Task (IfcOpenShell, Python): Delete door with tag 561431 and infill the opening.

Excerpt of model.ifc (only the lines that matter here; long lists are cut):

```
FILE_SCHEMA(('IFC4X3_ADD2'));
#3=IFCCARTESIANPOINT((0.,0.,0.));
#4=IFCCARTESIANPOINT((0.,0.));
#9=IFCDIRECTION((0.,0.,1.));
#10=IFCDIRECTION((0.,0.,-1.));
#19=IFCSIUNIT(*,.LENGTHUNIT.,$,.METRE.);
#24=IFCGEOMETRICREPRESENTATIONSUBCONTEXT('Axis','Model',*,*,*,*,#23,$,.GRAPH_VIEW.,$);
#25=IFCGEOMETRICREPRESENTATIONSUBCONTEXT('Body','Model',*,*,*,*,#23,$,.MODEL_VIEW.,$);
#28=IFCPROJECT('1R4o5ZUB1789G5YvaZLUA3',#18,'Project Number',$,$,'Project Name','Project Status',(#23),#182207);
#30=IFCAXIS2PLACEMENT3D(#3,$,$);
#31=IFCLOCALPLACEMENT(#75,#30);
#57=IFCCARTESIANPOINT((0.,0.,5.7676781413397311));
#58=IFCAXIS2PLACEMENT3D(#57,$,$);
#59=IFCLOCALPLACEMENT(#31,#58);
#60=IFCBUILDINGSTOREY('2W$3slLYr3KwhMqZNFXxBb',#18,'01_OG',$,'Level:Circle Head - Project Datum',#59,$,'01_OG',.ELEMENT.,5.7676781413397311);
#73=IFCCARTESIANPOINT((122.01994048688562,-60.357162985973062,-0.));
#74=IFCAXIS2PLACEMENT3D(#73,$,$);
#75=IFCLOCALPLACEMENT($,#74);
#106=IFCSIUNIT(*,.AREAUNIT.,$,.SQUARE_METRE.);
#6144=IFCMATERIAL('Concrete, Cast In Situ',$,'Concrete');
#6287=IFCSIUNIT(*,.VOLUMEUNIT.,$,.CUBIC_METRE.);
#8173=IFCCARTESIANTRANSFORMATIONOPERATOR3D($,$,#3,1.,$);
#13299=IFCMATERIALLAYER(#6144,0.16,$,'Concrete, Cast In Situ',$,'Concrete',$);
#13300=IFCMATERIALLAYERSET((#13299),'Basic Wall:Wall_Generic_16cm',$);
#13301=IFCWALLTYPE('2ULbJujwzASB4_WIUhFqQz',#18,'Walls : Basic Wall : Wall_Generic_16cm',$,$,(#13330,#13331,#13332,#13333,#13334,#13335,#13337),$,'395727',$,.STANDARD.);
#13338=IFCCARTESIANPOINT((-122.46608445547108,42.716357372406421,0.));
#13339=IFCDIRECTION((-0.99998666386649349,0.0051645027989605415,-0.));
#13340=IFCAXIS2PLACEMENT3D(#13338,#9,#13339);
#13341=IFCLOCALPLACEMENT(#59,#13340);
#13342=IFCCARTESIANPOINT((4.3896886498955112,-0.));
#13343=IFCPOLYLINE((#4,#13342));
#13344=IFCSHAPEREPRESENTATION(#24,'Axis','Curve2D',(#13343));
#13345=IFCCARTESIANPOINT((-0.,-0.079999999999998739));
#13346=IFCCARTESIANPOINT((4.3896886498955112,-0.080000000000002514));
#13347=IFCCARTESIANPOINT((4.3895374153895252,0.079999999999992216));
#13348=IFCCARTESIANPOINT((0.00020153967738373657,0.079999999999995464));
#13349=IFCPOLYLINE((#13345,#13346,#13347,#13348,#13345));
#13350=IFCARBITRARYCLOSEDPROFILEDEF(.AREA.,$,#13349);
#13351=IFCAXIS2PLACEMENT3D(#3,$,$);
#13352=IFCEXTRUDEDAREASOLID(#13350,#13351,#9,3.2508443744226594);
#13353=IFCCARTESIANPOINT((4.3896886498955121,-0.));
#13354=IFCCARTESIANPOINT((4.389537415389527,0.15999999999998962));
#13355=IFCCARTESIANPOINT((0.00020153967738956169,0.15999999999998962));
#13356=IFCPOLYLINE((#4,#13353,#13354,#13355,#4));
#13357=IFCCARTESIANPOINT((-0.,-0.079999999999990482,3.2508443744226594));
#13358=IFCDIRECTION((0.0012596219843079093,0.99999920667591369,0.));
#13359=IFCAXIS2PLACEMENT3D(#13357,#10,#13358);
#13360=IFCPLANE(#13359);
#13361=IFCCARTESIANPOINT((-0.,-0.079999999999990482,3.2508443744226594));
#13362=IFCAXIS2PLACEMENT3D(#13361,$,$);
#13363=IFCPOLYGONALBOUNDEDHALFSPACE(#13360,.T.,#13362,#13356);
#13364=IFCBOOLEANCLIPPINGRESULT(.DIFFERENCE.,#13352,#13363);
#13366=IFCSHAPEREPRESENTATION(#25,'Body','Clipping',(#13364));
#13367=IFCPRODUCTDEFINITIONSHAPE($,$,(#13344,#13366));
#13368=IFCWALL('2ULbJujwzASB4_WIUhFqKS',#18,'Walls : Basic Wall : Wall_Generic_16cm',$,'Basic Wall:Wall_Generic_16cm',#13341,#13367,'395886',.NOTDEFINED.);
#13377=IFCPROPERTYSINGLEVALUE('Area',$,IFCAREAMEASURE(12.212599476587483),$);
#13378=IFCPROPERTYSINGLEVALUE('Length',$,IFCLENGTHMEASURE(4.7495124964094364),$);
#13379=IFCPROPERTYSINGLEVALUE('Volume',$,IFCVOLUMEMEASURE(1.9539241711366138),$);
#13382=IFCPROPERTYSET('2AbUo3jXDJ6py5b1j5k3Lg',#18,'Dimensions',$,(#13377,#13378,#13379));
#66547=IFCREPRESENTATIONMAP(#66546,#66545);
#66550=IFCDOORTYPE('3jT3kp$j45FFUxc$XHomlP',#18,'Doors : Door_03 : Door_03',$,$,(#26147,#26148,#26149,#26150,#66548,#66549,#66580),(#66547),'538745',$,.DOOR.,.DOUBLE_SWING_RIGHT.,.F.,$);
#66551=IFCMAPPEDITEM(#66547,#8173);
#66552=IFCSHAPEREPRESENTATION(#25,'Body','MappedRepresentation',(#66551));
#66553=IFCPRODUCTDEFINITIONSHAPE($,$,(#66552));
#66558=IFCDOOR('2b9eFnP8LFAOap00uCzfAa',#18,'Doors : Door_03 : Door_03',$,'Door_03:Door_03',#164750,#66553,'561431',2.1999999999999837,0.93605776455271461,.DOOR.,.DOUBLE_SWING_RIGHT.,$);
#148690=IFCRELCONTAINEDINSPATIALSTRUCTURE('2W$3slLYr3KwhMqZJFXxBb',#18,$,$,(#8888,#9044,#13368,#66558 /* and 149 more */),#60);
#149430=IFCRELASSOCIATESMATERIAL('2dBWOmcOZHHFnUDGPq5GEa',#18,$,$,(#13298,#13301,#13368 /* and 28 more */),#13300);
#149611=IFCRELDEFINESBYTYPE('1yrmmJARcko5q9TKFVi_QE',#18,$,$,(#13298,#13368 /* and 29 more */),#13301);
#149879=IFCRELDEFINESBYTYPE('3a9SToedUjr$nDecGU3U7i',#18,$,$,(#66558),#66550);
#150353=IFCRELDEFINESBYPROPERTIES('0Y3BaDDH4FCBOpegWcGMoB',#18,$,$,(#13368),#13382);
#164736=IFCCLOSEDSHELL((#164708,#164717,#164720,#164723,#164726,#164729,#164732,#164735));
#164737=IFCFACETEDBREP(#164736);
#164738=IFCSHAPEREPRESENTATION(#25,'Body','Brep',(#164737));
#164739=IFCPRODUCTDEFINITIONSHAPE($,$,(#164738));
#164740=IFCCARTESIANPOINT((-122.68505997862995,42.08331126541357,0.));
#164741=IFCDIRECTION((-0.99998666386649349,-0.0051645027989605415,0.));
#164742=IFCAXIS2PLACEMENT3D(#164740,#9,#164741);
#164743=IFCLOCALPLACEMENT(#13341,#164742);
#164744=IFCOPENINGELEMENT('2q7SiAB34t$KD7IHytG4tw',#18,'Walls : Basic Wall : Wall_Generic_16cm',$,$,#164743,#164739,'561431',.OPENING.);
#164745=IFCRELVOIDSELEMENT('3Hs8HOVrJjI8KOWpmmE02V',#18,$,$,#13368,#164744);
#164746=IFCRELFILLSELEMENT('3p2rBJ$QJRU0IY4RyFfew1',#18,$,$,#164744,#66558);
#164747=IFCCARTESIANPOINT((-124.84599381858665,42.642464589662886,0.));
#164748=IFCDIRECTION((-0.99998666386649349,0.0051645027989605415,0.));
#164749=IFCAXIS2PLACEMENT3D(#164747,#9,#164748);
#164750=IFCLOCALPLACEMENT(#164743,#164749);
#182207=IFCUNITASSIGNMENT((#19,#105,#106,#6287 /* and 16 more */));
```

```python
import ifcopenshell
import ifcopenshell.api.feature
import ifcopenshell.api.pset
import ifcopenshell.api.root
import ifcopenshell.geom
import ifcopenshell.util.element
import ifcopenshell.util.shape
import ifcopenshell.util.unit

model = ifcopenshell.open("model.ifc")
area_scale = ifcopenshell.util.unit.calculate_unit_scale(model, "AREAUNIT")
volume_scale = ifcopenshell.util.unit.calculate_unit_scale(model, "VOLUMEUNIT")
settings = ifcopenshell.geom.settings()


def volume(element):
    """Net volume in cubic metres, openings subtracted."""
    shape = ifcopenshell.geom.create_shape(settings, element)
    return ifcopenshell.util.shape.get_volume(shape.geometry)


door = model.by_guid("2b9eFnP8LFAOap00uCzfAa")
opening = door.FillsVoids[0].RelatingOpeningElement
wall = opening.VoidsElements[0].RelatingBuildingElement
before = volume(wall)

ifcopenshell.api.root.remove_product(model, product=door)
ifcopenshell.api.feature.remove_feature(model, feature=opening)

after = volume(wall)
thickness = 0.16  # wall thickness in metres

# Update the wall's stored quantities.
pset = model.by_id(ifcopenshell.util.element.get_pset(wall, "Dimensions", should_inherit=False)["id"])
ifcopenshell.api.pset.edit_pset(model, pset=pset, properties={
    "Area": model.create_entity("IfcAreaMeasure", after / thickness / area_scale),
    "Volume": model.create_entity("IfcVolumeMeasure", after / volume_scale),
})

print(f"wall volume {before:.3f} -> {after:.3f} m3")

model.write("model_edited.ifc")
```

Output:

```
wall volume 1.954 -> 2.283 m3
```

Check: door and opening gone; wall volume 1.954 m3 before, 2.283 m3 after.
